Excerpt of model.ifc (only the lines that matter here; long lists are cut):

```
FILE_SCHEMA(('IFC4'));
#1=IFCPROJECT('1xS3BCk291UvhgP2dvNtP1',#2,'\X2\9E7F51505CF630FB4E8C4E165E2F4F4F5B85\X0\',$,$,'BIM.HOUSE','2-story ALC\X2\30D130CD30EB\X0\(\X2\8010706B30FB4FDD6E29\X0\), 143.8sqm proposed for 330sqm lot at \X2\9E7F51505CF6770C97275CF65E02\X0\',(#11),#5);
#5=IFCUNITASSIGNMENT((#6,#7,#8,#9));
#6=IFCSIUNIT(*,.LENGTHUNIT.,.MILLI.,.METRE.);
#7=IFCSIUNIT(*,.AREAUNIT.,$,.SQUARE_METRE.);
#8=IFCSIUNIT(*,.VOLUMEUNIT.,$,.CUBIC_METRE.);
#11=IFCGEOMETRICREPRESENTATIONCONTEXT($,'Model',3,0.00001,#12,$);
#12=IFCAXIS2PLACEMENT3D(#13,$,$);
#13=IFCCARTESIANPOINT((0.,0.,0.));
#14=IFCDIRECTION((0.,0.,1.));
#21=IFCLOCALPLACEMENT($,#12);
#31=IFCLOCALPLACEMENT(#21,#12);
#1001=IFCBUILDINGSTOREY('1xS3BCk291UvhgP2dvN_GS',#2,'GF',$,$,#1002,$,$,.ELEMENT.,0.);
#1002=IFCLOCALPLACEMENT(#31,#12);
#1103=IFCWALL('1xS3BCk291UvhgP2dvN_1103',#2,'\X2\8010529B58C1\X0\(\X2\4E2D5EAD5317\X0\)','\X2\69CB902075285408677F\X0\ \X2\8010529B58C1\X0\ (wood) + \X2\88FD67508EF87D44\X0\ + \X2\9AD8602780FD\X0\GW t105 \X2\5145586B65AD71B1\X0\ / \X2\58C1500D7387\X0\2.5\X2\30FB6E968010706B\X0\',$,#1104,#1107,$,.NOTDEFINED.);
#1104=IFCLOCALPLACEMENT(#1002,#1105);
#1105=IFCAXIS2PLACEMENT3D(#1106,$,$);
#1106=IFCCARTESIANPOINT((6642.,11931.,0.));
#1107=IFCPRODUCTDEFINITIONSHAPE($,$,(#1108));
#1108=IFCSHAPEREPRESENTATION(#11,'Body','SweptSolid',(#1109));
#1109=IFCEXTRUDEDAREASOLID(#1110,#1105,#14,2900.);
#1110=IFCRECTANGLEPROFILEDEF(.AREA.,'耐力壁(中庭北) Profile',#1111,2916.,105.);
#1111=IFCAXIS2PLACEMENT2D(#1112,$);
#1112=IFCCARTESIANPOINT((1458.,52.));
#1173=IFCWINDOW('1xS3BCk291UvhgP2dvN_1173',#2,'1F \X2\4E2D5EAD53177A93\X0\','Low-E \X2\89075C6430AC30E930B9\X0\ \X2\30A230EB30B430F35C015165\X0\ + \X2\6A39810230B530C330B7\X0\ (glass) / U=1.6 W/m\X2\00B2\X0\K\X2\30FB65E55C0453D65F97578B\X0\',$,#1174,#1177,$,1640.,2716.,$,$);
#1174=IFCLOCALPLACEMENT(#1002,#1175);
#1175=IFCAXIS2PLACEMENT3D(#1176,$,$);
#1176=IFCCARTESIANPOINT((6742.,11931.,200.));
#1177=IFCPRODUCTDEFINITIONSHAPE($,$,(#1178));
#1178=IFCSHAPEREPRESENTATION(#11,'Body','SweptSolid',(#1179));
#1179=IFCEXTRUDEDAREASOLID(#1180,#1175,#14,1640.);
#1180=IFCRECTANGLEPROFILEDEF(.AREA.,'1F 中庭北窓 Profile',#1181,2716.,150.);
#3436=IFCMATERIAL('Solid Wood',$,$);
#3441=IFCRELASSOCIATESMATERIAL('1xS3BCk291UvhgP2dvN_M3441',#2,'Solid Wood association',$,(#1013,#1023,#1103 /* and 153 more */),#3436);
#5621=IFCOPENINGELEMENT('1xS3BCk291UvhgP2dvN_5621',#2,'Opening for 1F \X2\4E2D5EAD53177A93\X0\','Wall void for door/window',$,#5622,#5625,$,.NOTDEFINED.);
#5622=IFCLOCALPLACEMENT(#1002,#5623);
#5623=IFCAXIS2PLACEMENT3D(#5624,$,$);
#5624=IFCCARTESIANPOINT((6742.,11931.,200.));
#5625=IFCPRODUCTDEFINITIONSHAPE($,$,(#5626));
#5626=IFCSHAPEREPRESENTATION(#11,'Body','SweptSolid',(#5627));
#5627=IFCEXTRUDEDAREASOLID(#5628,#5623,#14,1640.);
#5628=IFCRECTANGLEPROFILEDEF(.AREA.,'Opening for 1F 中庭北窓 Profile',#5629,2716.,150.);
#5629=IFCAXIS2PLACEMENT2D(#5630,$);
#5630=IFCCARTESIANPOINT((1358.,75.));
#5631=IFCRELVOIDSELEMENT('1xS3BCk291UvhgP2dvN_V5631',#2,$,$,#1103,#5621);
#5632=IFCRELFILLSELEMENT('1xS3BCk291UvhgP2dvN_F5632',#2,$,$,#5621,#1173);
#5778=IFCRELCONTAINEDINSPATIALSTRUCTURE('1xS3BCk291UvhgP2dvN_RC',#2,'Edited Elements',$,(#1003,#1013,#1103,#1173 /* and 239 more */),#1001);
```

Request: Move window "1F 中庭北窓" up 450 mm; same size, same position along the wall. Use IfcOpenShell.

```python
import numpy as np
import ifcopenshell
import ifcopenshell.api.geometry
import ifcopenshell.util.placement
import ifcopenshell.util.unit

model = ifcopenshell.open("model.ifc")
unit_scale = ifcopenshell.util.unit.calculate_unit_scale(model)

window = model.by_id(1173)
opening = window.FillsVoids[0].RelatingOpeningElement
dz = 0.45 / unit_scale

shift = np.array([0.0, 0.0, dz])
# The window is not placed relative to its opening, so move both.
for product in (opening, window):
    matrix = ifcopenshell.util.placement.get_local_placement(product.ObjectPlacement)
    matrix[:3, 3] += shift
    ifcopenshell.api.geometry.edit_object_placement(model, product=product, matrix=matrix, is_si=False)

print(f"moved by {dz * unit_scale:+.3f} m")

model.write("model-out.ifc")
```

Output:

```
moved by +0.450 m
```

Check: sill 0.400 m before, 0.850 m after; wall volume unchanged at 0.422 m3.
